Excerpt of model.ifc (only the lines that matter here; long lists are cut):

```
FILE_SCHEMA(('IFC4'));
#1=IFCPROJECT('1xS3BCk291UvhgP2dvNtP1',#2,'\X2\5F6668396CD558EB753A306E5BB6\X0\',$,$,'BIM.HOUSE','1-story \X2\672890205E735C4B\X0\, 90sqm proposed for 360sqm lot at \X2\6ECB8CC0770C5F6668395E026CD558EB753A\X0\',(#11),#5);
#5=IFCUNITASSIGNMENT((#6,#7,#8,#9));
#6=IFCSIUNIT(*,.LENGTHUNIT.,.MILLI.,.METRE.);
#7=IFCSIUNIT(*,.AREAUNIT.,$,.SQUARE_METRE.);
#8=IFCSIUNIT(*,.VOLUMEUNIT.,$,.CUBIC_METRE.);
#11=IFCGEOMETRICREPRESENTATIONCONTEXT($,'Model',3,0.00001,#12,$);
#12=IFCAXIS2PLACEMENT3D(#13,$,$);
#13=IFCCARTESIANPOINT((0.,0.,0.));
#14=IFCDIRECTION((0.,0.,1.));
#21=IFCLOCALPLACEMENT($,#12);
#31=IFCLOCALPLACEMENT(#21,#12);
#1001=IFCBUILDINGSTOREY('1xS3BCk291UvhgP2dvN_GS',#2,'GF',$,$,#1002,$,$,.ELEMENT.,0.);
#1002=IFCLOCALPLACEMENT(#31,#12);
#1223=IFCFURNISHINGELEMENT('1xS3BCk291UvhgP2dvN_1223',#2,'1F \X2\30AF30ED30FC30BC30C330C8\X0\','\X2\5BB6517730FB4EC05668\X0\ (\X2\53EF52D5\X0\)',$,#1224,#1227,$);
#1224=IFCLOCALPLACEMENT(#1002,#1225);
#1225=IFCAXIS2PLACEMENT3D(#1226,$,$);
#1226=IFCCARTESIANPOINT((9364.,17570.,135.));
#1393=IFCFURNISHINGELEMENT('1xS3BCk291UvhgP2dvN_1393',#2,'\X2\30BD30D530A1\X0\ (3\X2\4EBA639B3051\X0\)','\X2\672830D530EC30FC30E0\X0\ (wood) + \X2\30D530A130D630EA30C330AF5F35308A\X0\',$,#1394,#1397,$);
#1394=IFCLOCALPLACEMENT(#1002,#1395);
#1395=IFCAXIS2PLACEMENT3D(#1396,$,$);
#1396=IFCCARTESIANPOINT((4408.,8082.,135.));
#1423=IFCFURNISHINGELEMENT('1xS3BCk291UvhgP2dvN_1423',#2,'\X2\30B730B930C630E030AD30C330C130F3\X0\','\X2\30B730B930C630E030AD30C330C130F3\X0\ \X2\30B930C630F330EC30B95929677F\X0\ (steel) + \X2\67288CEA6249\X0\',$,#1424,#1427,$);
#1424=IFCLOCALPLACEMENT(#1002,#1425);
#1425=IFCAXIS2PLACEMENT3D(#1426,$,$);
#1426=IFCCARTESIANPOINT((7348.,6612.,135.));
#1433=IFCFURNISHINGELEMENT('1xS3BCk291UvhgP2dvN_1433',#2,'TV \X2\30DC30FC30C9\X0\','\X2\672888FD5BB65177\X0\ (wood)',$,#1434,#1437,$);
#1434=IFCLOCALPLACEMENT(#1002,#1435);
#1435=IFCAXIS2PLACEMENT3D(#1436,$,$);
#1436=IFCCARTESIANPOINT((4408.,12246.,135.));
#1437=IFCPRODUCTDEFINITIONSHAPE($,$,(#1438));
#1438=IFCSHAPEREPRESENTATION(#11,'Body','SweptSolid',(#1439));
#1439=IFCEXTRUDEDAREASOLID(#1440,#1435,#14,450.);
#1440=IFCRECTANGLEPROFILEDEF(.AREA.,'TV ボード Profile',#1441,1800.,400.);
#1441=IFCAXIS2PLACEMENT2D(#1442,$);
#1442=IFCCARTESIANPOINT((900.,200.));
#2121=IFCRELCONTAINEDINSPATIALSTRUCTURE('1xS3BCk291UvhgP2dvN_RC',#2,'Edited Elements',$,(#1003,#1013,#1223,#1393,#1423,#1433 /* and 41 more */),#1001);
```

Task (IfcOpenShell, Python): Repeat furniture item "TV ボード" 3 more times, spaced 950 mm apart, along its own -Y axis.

```python
import ifcopenshell
import ifcopenshell.api.geometry
import ifcopenshell.api.root
import ifcopenshell.util.element
import ifcopenshell.util.placement

model = ifcopenshell.open("model.ifc")


def reuse_history(source, copy):
    """copy_class also copies each property set's owner history, people and application; keep the originals."""
    for rel in copy.IsDefinedBy:
        if rel.is_a("IfcRelDefinesByProperties") and (history := rel.RelatingPropertyDefinition.OwnerHistory):
            rel.RelatingPropertyDefinition.OwnerHistory = source.OwnerHistory
            ifcopenshell.util.element.remove_deep2(model, history)


source = model.by_guid("1xS3BCk291UvhgP2dvN_1433")
base = ifcopenshell.util.placement.get_local_placement(source.ObjectPlacement)
step = -base[:3, 1] * 950.0

for i in range(1, 4):
    copy = ifcopenshell.api.root.copy_class(model, product=source)
    copy.Representation = ifcopenshell.util.element.copy_deep(
        model, source.Representation, exclude=["IfcGeometricRepresentationContext", "IfcRepresentationMap"]
    )
    reuse_history(source, copy)
    matrix = base.copy()
    matrix[:3, 3] += i * step
    print("added at", matrix[:3, 3].round(3) + 0.0)
    ifcopenshell.api.geometry.edit_object_placement(model, product=copy, matrix=matrix, is_si=False)

model.write("model_rev.ifc")
```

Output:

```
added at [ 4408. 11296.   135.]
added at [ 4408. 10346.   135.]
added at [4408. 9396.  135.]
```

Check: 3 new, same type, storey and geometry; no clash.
